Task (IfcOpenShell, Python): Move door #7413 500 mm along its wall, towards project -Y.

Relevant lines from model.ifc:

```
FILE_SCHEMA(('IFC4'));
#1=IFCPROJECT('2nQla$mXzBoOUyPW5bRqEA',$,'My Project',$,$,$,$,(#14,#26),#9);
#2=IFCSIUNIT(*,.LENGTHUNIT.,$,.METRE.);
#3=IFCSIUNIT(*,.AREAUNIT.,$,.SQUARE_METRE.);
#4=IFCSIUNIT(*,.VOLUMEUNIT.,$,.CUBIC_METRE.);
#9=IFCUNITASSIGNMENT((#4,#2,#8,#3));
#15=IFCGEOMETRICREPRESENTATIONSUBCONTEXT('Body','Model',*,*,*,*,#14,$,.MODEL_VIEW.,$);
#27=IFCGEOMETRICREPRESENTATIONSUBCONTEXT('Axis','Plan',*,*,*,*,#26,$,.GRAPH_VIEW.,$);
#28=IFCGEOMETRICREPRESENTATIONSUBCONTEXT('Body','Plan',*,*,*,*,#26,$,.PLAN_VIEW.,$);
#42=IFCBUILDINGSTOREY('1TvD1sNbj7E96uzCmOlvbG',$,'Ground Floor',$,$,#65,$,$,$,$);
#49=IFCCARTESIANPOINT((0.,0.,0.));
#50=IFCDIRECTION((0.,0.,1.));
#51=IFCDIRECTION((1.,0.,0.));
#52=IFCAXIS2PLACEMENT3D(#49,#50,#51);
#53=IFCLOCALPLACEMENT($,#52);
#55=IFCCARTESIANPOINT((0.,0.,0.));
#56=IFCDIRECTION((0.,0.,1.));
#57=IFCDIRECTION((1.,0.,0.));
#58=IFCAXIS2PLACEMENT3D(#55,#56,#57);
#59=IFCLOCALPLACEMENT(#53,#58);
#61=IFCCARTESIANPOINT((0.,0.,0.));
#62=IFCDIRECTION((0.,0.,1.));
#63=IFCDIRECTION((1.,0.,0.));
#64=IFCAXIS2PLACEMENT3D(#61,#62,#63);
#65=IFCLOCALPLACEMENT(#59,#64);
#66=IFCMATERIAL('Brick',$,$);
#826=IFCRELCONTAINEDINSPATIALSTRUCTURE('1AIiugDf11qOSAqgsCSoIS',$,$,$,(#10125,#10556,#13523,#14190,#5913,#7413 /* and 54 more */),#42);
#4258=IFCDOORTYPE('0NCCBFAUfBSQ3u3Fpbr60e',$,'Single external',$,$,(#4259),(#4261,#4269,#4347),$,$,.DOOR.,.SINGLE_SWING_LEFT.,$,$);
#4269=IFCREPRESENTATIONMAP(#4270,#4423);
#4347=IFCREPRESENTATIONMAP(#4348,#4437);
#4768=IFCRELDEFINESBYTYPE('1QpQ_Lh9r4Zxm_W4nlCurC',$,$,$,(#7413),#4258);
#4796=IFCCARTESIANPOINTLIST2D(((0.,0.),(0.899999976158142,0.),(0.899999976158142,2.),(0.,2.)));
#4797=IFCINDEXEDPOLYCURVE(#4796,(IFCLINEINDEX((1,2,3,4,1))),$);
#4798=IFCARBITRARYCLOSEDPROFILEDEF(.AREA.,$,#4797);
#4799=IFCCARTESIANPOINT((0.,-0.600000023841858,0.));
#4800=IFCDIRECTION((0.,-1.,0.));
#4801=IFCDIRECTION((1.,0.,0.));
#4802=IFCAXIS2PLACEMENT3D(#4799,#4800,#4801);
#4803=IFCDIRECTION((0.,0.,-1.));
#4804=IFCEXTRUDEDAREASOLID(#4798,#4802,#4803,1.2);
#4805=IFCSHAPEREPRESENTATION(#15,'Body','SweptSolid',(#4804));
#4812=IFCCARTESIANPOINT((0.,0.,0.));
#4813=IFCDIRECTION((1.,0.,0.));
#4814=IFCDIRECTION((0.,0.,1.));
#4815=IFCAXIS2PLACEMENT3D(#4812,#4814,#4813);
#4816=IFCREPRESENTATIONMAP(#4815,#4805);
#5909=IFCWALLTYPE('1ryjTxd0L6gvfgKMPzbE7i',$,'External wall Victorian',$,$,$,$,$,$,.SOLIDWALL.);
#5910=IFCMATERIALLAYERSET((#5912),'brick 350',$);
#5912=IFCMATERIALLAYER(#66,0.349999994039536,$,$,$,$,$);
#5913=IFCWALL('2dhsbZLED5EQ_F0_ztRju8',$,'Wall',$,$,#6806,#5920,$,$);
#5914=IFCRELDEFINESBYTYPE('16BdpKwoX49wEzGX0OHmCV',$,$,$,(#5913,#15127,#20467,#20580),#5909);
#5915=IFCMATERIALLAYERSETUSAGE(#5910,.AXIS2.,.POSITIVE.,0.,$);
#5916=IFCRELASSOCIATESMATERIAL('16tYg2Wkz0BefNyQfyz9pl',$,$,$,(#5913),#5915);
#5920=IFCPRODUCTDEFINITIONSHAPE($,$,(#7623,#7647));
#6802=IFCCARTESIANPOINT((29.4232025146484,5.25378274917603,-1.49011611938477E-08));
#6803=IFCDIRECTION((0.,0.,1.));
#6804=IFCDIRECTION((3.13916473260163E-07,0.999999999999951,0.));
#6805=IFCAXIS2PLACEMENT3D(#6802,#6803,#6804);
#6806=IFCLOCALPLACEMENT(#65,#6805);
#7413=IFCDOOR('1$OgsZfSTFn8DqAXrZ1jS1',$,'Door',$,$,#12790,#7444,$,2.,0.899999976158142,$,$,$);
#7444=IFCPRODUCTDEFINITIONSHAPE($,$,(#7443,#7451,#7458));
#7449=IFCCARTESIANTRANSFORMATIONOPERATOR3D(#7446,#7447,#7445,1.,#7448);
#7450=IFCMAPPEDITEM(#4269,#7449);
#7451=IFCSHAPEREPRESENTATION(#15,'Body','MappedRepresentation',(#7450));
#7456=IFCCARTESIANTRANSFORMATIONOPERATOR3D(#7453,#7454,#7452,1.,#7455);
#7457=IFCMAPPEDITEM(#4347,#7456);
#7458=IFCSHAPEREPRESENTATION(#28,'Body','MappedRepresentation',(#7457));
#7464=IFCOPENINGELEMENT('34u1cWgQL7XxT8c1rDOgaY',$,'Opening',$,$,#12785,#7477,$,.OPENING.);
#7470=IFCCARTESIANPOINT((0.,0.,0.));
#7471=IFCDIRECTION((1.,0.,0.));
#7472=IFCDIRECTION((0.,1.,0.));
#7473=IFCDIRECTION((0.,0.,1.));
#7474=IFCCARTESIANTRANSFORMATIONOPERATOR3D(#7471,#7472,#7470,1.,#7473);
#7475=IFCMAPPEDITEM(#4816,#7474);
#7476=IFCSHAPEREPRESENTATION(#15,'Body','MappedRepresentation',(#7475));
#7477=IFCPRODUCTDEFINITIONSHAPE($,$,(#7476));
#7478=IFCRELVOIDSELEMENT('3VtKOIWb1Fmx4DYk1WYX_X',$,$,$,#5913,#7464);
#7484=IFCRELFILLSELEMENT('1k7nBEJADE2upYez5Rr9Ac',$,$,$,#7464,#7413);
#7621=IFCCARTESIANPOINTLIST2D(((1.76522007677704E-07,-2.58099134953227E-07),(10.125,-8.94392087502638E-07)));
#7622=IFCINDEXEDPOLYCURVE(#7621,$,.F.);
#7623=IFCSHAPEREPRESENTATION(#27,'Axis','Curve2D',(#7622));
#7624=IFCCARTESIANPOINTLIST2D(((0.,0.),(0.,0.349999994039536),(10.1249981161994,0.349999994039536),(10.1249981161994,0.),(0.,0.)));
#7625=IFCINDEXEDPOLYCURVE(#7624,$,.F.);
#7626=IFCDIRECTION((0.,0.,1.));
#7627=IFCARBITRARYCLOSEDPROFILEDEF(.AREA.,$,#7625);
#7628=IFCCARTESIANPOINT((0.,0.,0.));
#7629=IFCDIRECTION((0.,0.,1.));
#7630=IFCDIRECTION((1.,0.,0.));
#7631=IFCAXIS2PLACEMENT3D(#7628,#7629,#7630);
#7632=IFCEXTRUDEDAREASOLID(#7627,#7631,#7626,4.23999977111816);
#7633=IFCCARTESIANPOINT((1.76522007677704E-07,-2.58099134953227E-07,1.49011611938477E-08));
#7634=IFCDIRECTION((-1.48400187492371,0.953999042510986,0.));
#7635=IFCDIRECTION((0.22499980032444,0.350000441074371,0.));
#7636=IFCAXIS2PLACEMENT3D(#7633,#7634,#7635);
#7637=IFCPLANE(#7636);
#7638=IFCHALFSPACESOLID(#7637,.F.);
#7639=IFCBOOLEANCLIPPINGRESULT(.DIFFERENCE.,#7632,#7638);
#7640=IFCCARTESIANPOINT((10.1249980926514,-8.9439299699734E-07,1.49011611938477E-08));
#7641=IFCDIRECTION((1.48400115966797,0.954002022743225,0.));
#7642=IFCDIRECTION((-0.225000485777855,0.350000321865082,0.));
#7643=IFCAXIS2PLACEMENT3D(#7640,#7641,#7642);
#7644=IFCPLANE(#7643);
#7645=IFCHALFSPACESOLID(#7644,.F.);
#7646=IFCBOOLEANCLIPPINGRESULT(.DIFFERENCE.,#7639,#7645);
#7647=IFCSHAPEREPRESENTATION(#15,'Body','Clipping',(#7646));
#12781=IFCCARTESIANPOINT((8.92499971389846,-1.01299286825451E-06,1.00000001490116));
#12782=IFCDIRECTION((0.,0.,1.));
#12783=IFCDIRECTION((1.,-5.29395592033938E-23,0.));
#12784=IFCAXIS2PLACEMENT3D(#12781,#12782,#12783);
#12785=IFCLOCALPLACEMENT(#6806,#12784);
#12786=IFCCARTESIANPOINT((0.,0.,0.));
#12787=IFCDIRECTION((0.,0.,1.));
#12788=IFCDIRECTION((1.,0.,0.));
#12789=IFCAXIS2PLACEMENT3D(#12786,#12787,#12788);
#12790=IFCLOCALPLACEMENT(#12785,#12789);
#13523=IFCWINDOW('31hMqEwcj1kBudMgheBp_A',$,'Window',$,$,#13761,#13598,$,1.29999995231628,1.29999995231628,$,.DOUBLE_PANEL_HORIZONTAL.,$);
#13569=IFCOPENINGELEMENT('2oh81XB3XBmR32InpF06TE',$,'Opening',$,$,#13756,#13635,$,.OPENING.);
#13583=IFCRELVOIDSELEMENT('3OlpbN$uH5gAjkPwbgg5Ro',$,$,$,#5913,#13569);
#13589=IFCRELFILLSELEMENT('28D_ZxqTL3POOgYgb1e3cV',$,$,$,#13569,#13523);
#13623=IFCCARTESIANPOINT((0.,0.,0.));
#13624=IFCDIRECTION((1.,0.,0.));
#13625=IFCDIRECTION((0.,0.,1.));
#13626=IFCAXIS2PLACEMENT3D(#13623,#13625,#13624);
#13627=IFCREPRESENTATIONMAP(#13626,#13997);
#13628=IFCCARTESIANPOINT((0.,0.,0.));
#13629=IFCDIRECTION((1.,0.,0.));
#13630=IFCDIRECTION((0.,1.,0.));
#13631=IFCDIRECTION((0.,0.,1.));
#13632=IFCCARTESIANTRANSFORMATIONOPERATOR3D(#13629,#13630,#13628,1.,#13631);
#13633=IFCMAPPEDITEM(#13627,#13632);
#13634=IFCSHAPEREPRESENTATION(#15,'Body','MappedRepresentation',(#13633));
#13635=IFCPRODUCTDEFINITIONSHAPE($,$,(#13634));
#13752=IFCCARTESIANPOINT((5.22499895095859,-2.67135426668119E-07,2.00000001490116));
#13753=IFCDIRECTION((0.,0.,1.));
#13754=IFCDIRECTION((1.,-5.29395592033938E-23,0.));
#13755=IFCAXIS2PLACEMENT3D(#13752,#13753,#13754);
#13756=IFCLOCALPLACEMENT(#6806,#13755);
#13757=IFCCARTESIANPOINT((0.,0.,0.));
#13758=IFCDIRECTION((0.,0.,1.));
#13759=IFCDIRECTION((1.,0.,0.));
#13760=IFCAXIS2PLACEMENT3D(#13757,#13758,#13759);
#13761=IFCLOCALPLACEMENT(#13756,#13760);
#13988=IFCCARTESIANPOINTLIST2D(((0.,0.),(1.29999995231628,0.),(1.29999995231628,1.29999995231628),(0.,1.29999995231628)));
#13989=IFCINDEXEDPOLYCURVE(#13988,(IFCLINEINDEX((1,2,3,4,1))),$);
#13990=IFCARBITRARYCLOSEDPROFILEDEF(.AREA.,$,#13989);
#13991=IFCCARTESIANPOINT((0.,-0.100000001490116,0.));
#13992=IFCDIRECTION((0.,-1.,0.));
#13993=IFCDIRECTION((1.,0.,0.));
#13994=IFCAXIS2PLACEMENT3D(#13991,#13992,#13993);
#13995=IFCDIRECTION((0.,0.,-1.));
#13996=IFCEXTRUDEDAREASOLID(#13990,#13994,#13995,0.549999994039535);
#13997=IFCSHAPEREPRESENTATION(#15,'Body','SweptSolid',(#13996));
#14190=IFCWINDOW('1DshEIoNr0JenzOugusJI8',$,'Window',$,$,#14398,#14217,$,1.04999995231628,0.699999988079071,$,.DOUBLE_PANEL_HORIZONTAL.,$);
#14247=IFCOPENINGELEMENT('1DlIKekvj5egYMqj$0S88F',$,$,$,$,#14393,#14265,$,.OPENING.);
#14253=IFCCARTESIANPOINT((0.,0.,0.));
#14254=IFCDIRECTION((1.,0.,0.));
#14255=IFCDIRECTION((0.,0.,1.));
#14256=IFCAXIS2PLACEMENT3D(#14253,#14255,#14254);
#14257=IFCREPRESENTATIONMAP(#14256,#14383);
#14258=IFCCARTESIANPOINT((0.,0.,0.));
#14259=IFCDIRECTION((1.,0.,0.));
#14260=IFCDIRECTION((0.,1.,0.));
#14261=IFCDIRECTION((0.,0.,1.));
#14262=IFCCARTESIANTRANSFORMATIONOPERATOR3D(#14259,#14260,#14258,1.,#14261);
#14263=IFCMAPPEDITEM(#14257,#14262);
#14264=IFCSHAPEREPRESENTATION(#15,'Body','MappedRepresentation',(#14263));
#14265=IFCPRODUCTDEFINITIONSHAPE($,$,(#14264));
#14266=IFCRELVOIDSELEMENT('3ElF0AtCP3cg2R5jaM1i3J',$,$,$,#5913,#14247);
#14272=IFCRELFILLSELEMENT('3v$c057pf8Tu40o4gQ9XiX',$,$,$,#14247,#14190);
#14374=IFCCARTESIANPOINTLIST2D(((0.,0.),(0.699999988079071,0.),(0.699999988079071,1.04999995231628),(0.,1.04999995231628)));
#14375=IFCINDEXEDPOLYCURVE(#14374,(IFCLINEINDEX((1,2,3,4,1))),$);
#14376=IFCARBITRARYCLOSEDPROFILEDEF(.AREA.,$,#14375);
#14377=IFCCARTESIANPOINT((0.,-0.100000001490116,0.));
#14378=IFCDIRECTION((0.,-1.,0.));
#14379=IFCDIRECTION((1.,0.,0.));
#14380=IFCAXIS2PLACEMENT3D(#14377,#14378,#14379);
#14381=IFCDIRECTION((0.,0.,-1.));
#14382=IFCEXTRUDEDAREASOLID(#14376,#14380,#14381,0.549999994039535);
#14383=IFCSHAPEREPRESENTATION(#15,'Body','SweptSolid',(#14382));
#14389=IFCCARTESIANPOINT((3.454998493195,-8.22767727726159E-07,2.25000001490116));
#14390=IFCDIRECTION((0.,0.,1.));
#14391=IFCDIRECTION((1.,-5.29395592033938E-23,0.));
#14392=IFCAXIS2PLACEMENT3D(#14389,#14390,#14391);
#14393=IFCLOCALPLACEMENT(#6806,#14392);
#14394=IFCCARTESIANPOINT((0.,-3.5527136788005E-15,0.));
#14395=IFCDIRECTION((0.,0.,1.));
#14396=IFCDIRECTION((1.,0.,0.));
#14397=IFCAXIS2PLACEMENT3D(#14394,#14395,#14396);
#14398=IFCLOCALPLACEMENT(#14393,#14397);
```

```python
import ifcopenshell
import ifcopenshell.api.geometry
import ifcopenshell.util.placement
import ifcopenshell.util.unit

model = ifcopenshell.open("model.ifc")
unit_scale = ifcopenshell.util.unit.calculate_unit_scale(model)

door = model.by_id(7413)
opening = door.FillsVoids[0].RelatingOpeningElement
wall = opening.VoidsElements[0].RelatingBuildingElement

wall_matrix = ifcopenshell.util.placement.get_local_placement(wall.ObjectPlacement)
shift = wall_matrix[:3, 0] * -0.5 / unit_scale
before = ifcopenshell.util.placement.get_local_placement(door.ObjectPlacement)[:3, 3].copy()

# The door is placed relative to its opening, so it follows when the opening moves.
matrix = ifcopenshell.util.placement.get_local_placement(opening.ObjectPlacement)
matrix[:3, 3] += shift
ifcopenshell.api.geometry.edit_object_placement(
    model, product=opening, matrix=matrix, is_si=False, should_transform_children=True
)

after = ifcopenshell.util.placement.get_local_placement(door.ObjectPlacement)[:3, 3]
print("door moved by", (after - before).round(3) + 0.0)

model.write("model_rev.ifc")
```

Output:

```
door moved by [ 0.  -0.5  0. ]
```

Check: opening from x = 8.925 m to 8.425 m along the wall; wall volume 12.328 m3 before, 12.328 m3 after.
